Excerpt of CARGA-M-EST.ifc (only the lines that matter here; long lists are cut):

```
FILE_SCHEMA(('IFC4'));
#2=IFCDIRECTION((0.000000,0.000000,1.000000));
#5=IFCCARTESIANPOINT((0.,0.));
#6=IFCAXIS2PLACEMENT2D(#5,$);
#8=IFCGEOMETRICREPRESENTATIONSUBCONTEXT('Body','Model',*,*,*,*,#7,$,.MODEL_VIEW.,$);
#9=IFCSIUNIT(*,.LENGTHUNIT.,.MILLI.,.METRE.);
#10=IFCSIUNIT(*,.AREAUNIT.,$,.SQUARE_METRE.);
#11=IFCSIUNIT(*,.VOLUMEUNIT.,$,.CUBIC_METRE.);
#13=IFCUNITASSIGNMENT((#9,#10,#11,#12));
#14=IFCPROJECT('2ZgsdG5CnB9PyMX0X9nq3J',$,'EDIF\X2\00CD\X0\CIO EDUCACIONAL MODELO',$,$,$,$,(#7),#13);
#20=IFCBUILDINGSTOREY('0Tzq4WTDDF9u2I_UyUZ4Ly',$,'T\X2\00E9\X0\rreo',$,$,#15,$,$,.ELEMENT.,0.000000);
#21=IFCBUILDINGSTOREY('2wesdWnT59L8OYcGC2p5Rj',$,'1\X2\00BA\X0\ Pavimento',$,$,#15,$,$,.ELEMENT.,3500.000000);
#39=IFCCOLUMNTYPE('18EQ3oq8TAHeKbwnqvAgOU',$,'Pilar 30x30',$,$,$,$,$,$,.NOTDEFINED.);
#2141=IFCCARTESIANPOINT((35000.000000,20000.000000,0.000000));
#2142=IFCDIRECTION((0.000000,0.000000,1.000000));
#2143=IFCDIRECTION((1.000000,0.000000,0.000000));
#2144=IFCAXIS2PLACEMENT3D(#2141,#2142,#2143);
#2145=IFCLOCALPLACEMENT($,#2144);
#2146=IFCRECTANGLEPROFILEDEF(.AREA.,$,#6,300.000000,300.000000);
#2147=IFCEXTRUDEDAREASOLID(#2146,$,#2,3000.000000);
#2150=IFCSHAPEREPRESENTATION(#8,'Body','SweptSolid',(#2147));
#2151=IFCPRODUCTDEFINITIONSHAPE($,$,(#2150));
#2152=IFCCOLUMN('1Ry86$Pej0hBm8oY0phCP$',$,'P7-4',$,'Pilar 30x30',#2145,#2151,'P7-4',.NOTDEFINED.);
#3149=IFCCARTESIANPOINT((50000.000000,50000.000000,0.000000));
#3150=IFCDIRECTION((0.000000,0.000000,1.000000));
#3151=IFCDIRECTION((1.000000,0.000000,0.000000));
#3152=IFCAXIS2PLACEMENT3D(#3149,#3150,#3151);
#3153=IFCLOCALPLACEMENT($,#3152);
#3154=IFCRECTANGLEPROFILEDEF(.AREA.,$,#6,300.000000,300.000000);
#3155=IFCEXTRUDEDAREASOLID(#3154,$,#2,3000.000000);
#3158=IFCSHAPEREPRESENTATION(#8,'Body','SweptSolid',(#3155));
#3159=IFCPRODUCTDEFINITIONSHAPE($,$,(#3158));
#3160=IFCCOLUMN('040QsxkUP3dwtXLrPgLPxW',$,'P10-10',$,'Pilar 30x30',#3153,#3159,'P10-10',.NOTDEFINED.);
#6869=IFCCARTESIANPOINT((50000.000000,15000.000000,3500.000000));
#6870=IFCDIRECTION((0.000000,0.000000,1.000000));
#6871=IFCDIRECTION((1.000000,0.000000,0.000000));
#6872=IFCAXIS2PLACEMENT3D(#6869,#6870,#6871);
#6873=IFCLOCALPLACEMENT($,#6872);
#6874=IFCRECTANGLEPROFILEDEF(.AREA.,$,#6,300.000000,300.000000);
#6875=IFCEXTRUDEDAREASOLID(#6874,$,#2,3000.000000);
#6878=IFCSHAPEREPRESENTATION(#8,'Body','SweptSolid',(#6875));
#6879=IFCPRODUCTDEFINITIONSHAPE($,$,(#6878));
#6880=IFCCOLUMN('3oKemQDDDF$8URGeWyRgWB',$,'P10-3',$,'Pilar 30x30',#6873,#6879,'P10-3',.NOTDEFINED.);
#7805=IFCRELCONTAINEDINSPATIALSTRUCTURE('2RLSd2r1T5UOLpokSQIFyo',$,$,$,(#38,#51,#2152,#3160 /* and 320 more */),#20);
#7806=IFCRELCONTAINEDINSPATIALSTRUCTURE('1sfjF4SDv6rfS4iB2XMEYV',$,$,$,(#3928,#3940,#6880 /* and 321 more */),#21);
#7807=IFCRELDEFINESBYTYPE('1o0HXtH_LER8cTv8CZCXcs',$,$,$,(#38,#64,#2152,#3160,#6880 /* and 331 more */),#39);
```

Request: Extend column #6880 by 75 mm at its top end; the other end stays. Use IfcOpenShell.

```python
import ifcopenshell
import ifcopenshell.util.representation

model = ifcopenshell.open("CARGA-M-EST.ifc")

member = model.by_id(6880)
change = 75.0

# The extrusion runs towards the end named, so only its depth changes.
body = ifcopenshell.util.representation.get_representation(member, "Model", "Body")
solid = body.Items[0]
old_length = solid.Depth
solid.Depth += change

print(f"length {old_length:g} -> {solid.Depth:g}")

model.write("CARGA-M-EST-out.ifc")
```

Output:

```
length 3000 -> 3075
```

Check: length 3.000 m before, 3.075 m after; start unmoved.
